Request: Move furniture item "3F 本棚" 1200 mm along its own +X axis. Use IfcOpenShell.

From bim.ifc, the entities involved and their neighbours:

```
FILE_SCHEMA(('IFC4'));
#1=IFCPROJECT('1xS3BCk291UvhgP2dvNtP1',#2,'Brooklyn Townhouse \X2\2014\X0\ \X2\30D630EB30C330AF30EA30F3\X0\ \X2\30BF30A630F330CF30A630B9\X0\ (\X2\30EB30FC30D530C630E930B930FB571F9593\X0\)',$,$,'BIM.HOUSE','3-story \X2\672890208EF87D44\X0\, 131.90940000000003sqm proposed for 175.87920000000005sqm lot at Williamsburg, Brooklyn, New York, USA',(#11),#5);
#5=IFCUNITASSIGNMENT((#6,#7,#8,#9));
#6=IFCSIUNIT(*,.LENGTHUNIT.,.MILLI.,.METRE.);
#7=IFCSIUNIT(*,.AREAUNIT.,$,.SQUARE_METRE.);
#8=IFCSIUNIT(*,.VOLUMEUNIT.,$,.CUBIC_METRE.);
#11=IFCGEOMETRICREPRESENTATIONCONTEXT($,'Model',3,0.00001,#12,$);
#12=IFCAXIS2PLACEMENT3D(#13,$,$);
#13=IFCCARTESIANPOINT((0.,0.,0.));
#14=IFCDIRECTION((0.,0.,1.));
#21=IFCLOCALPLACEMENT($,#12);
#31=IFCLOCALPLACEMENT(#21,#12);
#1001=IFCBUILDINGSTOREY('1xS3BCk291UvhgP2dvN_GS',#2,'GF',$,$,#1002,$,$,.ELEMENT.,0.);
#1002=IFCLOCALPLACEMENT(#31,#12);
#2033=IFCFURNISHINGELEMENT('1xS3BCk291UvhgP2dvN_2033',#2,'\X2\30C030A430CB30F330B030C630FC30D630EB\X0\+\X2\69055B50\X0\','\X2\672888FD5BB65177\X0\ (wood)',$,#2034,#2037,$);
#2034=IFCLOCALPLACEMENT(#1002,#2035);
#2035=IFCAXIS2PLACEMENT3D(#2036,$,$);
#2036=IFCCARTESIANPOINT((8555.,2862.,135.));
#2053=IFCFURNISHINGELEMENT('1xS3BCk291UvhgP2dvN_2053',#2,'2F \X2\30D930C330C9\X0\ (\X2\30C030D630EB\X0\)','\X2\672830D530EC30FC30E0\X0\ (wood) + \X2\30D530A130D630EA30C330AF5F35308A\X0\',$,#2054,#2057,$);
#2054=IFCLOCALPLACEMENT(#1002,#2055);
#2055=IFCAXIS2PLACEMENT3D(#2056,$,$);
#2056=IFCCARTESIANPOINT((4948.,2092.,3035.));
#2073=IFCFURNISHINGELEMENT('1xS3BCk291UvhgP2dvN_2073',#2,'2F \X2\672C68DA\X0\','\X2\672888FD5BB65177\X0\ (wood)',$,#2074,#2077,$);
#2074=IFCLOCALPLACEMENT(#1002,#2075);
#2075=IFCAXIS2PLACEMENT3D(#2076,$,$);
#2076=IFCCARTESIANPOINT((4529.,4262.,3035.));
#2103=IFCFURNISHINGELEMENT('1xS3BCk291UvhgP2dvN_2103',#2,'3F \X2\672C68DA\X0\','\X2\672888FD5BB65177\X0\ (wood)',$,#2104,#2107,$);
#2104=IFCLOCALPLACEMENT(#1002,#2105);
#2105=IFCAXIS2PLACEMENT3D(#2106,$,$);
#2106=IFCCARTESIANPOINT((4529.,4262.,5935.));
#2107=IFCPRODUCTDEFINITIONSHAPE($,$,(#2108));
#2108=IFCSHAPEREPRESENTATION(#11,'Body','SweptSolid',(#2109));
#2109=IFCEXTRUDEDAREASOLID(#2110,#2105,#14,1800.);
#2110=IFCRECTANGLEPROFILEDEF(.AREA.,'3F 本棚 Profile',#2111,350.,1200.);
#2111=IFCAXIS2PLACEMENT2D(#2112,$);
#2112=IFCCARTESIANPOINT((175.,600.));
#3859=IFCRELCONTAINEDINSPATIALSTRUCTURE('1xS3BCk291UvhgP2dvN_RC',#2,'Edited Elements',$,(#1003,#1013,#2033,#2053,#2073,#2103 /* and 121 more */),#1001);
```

```python
import ifcopenshell
import ifcopenshell.api.geometry
import ifcopenshell.util.placement
import ifcopenshell.util.unit

model = ifcopenshell.open("bim.ifc")
unit_scale = ifcopenshell.util.unit.calculate_unit_scale(model)

item = model.by_guid("1xS3BCk291UvhgP2dvN_2103")
matrix = ifcopenshell.util.placement.get_local_placement(item.ObjectPlacement)
matrix[:3, 3] += matrix[:3, 0] * 1.2 / unit_scale
ifcopenshell.api.geometry.edit_object_placement(model, product=item, matrix=matrix, is_si=False)

print(ifcopenshell.util.placement.get_local_placement(item.ObjectPlacement).round(3) + 0.0)

model.write("bim_rev.ifc")
```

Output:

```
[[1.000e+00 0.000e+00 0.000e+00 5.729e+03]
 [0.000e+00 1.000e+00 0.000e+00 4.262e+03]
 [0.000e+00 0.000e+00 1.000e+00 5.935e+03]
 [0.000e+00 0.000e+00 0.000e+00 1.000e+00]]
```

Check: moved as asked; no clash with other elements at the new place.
